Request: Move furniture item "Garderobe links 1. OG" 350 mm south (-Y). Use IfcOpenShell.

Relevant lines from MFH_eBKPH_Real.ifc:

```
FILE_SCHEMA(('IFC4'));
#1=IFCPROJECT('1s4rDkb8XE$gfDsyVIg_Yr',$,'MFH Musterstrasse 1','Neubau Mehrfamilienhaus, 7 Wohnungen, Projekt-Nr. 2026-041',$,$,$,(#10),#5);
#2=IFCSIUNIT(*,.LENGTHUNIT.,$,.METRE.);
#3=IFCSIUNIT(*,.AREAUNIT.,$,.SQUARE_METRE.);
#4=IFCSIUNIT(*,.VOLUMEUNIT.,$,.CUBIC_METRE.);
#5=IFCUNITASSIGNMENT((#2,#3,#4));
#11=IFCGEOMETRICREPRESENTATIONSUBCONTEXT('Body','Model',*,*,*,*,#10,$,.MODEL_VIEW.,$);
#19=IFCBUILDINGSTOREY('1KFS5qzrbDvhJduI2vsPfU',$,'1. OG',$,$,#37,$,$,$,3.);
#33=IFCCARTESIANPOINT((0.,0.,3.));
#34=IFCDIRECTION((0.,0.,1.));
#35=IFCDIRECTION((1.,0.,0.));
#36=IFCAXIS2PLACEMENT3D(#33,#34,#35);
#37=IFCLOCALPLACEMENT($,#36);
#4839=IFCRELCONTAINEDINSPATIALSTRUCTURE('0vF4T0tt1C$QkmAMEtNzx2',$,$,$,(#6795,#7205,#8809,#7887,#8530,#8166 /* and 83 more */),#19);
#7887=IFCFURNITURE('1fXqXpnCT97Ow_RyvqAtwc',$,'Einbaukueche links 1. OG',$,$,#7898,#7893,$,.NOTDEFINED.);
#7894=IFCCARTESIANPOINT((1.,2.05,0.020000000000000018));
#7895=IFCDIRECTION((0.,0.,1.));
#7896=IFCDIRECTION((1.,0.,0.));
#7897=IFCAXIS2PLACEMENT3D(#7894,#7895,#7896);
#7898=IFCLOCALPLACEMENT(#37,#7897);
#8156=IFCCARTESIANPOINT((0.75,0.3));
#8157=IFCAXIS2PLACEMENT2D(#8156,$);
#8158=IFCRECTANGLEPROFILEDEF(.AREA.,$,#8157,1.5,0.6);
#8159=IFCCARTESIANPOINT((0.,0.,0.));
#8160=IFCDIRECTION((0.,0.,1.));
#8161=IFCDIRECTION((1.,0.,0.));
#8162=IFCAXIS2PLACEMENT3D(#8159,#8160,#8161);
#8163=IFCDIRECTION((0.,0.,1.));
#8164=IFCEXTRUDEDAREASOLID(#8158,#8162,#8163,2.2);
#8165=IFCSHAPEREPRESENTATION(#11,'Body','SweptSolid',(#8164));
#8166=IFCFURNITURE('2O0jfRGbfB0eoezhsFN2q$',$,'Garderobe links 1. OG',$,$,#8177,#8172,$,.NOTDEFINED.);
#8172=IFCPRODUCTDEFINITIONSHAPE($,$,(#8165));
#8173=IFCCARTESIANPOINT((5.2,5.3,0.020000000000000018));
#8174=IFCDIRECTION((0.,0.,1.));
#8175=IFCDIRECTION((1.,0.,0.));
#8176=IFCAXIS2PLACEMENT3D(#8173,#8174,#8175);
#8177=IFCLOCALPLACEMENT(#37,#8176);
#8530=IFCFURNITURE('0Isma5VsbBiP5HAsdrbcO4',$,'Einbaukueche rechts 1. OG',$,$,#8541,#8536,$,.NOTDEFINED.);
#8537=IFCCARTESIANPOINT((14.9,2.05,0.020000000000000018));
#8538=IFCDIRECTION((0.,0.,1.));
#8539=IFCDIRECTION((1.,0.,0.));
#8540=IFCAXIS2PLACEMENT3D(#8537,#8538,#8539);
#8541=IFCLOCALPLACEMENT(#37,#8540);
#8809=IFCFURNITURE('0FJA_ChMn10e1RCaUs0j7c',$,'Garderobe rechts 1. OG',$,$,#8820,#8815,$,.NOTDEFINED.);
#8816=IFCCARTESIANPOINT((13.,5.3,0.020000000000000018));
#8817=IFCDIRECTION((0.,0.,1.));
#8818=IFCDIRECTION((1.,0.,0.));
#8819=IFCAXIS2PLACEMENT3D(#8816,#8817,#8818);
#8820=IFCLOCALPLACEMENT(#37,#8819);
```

```python
import ifcopenshell
import ifcopenshell.api.geometry
import ifcopenshell.util.placement

model = ifcopenshell.open("MFH_eBKPH_Real.ifc")

item = model.by_guid("2O0jfRGbfB0eoezhsFN2q$")
matrix = ifcopenshell.util.placement.get_local_placement(item.ObjectPlacement)
matrix[1, 3] -= 0.35
ifcopenshell.api.geometry.edit_object_placement(model, product=item, matrix=matrix, is_si=False)

print(ifcopenshell.util.placement.get_local_placement(item.ObjectPlacement).round(3) + 0.0)

model.write("MFH_eBKPH_Real-out.ifc")
```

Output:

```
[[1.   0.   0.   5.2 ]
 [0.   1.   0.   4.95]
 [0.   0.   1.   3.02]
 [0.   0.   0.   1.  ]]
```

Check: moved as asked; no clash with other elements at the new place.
